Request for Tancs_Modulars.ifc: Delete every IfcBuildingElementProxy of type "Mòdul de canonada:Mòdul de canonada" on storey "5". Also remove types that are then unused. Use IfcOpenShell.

First a look at what the model holds.

```python
import ifcopenshell
import ifcopenshell.util.element

model = ifcopenshell.open("Tancs_Modulars.ifc")
print(model.schema)
storey = next(s for s in model.by_type("IfcBuildingStorey") if s.Name == "5")
proxies = [e for e in ifcopenshell.util.element.get_decomposition(storey) if e.is_a("IfcBuildingElementProxy")]
seen = {}
for e in proxies:
    element_type = ifcopenshell.util.element.get_type(e)
    name = element_type.Name if element_type not in (None, e) else None
    seen[name] = seen.get(name, 0) + 1
for name, count in sorted(seen.items(), key=str):
    print(count, "x", name)
```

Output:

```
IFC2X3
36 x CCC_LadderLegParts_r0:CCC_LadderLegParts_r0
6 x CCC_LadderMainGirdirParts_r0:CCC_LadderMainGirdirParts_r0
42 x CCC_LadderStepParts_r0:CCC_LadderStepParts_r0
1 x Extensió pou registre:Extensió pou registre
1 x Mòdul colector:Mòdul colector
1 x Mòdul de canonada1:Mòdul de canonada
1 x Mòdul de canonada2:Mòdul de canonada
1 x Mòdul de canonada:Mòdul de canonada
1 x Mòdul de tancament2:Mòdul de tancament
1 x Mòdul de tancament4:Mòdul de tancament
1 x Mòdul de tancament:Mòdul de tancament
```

```python
import ifcopenshell
import ifcopenshell.api.root
import ifcopenshell.util.element

model = ifcopenshell.open("Tancs_Modulars.ifc")

storey = next(s for s in model.by_type("IfcBuildingStorey") if s.Name == "5")
proxies = [e for e in ifcopenshell.util.element.get_decomposition(storey) if e.is_a("IfcBuildingElementProxy")]
targets = [e for e in proxies if (t := ifcopenshell.util.element.get_type(e)) not in (None, e) and t.Name == "Mòdul de canonada:Mòdul de canonada"]
types = {ifcopenshell.util.element.get_type(e) for e in targets} - {None, *targets}

for e in targets:
    ifcopenshell.api.root.remove_product(model, product=e)
print(len(targets), "removed")

unused = [t for t in types if not ifcopenshell.util.element.get_types(t)]
for t in unused:
    ifcopenshell.api.root.remove_product(model, product=t)
print(len(unused), "unused types removed")

model.write("Tancs_Modulars-out.ifc")
```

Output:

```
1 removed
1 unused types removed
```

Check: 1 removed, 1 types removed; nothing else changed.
